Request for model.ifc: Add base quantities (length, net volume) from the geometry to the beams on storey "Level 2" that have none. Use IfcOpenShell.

First a look at what the model holds.

```python
import ifcopenshell
import ifcopenshell.util.element
import ifcopenshell.util.unit

model = ifcopenshell.open("model.ifc")
print(model.schema)
for unit_type in ("LENGTHUNIT", "AREAUNIT", "VOLUMEUNIT"):
    print(unit_type, ifcopenshell.util.unit.calculate_unit_scale(model, unit_type))
storey = next(s for s in model.by_type("IfcBuildingStorey") if s.Name == "Level 2")
beams = [e for e in ifcopenshell.util.element.get_decomposition(storey) if e.is_a("IfcBeam")]
for e in sorted(beams, key=lambda e: e.id()):
    print(e.id(), e.is_a(), e.Name, list(ifcopenshell.util.element.get_psets(e, qtos_only=True)), sep=" | ")
```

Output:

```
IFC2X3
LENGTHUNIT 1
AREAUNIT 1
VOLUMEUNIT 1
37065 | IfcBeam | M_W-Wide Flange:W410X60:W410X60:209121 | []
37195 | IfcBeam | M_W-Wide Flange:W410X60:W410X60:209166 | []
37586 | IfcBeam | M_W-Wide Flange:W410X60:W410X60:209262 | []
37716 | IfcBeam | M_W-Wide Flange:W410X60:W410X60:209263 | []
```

```python
import ifcopenshell
import ifcopenshell.api.pset
import ifcopenshell.geom
import ifcopenshell.util.element
import ifcopenshell.util.shape
import ifcopenshell.util.unit

model = ifcopenshell.open("model.ifc")
unit_scale = ifcopenshell.util.unit.calculate_unit_scale(model)
volume_scale = ifcopenshell.util.unit.calculate_unit_scale(model, "VOLUMEUNIT")
settings = ifcopenshell.geom.settings()

storey = next(s for s in model.by_type("IfcBuildingStorey") if s.Name == "Level 2")
beams = [e for e in ifcopenshell.util.element.get_decomposition(storey) if e.is_a("IfcBeam")]

for e in sorted(beams, key=lambda e: e.id()):
    if ifcopenshell.util.element.get_psets(e, qtos_only=True, should_inherit=False):
        continue
    # Geometry comes back in metres, in the element's own axes.
    shape = ifcopenshell.geom.create_shape(settings, e)
    values = {
        "Length": ifcopenshell.util.shape.get_max_xyz(shape.geometry) / unit_scale,
        "NetVolume": ifcopenshell.util.shape.get_volume(shape.geometry) / volume_scale,
    }
    qto = ifcopenshell.api.pset.add_qto(model, product=e, name="BaseQuantities")
    ifcopenshell.api.pset.edit_qto(model, qto=qto, properties=values)
    print(e.id(), {k: round(v, 3) for k, v in values.items()})

model.write("model_rev.ifc")
```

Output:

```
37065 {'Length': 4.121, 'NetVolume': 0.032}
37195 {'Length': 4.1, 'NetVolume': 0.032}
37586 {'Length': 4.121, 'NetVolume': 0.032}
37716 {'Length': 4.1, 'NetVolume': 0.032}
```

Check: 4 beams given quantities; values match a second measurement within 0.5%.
